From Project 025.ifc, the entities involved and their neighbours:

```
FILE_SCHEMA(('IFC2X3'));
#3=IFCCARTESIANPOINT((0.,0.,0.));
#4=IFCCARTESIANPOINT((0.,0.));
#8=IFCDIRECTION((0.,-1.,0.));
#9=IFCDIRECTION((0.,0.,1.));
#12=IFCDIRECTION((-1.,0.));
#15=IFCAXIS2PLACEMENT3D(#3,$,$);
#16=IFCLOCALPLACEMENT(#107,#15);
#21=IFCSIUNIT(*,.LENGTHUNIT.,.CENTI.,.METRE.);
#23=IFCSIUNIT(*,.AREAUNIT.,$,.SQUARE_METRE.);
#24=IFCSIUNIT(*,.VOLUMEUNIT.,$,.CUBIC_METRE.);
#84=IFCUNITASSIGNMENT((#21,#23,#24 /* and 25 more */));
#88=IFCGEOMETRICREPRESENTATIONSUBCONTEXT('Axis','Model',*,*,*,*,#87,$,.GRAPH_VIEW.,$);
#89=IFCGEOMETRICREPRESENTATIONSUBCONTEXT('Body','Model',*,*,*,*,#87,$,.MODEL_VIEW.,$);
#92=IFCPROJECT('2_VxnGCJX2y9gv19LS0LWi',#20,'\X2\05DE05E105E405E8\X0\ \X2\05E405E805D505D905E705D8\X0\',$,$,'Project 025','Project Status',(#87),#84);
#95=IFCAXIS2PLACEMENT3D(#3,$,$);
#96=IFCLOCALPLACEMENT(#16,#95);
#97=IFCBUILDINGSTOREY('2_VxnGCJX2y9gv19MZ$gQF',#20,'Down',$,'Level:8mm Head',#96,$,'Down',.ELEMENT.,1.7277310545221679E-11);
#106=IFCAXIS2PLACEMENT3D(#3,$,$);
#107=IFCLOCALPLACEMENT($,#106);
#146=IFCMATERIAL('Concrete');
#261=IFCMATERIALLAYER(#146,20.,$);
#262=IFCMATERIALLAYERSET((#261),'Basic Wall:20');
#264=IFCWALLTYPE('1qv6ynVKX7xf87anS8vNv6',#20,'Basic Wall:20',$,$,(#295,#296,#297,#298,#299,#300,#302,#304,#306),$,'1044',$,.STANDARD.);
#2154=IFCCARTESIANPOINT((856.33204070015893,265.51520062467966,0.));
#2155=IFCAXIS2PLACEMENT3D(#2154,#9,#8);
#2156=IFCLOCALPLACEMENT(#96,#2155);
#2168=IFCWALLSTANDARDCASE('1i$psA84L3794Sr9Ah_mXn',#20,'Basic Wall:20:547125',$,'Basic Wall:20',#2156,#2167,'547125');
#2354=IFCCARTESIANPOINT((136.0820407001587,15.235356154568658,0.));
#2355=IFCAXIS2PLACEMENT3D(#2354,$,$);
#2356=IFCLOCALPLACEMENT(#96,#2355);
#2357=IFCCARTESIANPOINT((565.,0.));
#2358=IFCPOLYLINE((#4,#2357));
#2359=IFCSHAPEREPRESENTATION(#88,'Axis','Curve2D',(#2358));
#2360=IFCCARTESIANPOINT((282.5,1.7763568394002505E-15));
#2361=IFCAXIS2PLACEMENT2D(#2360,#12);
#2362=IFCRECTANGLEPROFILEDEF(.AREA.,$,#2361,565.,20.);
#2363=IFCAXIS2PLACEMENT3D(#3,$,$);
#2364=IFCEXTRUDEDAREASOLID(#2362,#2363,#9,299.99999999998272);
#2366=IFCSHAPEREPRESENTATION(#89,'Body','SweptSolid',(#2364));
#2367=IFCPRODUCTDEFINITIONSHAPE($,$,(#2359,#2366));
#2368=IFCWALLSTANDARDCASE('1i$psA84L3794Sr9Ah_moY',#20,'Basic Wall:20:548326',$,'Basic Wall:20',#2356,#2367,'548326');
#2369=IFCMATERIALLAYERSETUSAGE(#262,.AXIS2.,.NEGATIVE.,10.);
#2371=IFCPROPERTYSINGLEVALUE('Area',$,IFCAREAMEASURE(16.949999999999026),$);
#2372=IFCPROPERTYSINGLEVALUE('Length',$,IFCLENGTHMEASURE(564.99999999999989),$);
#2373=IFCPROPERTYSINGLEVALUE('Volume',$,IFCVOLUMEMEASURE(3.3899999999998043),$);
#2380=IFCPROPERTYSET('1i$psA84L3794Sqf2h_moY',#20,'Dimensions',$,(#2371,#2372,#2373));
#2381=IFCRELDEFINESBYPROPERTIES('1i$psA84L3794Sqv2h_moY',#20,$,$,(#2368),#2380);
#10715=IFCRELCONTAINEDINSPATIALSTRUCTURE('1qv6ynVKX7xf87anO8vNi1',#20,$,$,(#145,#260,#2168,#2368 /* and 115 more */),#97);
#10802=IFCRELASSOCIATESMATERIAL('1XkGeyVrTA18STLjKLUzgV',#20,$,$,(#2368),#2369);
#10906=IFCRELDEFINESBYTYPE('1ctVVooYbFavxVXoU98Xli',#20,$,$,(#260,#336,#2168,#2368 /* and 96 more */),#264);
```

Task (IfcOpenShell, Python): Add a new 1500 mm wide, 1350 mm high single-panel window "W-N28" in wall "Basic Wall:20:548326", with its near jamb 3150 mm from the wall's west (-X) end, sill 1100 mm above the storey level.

```python
import numpy as np
import ifcopenshell
import ifcopenshell.api.feature
import ifcopenshell.api.geometry
import ifcopenshell.api.pset
import ifcopenshell.api.root
import ifcopenshell.api.spatial
import ifcopenshell.api.type
import ifcopenshell.geom
import ifcopenshell.util.element
import ifcopenshell.util.placement
import ifcopenshell.util.representation
import ifcopenshell.util.shape
import ifcopenshell.util.unit

model = ifcopenshell.open("Project 025.ifc")
unit_scale = ifcopenshell.util.unit.calculate_unit_scale(model)
area_scale = ifcopenshell.util.unit.calculate_unit_scale(model, "AREAUNIT")
volume_scale = ifcopenshell.util.unit.calculate_unit_scale(model, "VOLUMEUNIT")
settings = ifcopenshell.geom.settings()


def volume(element):
    """Net volume in cubic metres, openings subtracted."""
    shape = ifcopenshell.geom.create_shape(settings, element)
    return ifcopenshell.util.shape.get_volume(shape.geometry)


wall = model.by_id(2368)
storey = ifcopenshell.util.element.get_container(wall, ifc_class="IfcBuildingStorey")
context = ifcopenshell.util.representation.get_context(model, "Model", "Body", "MODEL_VIEW")
before = volume(wall)

width, height, from_end, sill = 1.5, 1.35, 3.15, 1.1  # metres

# The wall runs along its own X axis, and the end named is its -X end.
wall_shape = ifcopenshell.geom.create_shape(settings, wall)
x, y, z = ifcopenshell.util.shape.get_vertices(wall_shape.geometry).T
start = x.min() + from_end
face, thickness = float(y.min()), float(y.max() - y.min())
wall_matrix = ifcopenshell.util.placement.get_local_placement(wall.ObjectPlacement)
level = ifcopenshell.util.placement.get_local_placement(storey.ObjectPlacement)[2, 3]


def in_wall(x, y):
    """Placement at x, y metres in the wall's axes, at sill height."""
    matrix = wall_matrix.copy()
    matrix[:, 3] = wall_matrix @ np.array([x / unit_scale, y / unit_scale, 0.0, 1.0])
    matrix[2, 3] = level + sill / unit_scale
    return matrix


# Opening: a box that overshoots both wall faces by 50 mm.
opening = ifcopenshell.api.root.create_entity(model, ifc_class="IfcOpeningElement")
box = ifcopenshell.api.geometry.add_wall_representation(
    model, context=context, length=width, height=height, thickness=thickness + 0.1
)
ifcopenshell.api.geometry.assign_representation(model, product=opening, representation=box)
ifcopenshell.api.geometry.edit_object_placement(model, product=opening, matrix=in_wall(start, face - 0.05), is_si=False)
ifcopenshell.api.feature.add_feature(model, feature=opening, element=wall)

window = ifcopenshell.api.root.create_entity(model, ifc_class="IfcWindow", name="W-N28")
window.OverallWidth, window.OverallHeight = width / unit_scale, height / unit_scale
body = ifcopenshell.api.geometry.add_window_representation(
    model,
    context=context,
    overall_width=window.OverallWidth,
    overall_height=window.OverallHeight,
    partition_type="SINGLE_PANEL",
)
ifcopenshell.api.geometry.assign_representation(model, product=window, representation=body)
ifcopenshell.api.spatial.assign_container(model, products=[window], relating_structure=storey)
fills = ifcopenshell.api.feature.add_filling(model, opening=opening, element=window)
fills.OwnerHistory = window.OwnerHistory  # required in IFC2X3

# IFC2X3 keeps the operation on the window style.
style = ifcopenshell.api.root.create_entity(model, ifc_class="IfcWindowStyle", name="W-N28")
style.OperationType, style.ConstructionType = "SINGLE_PANEL", "NOTDEFINED"
style.ParameterTakesPrecedence = style.Sizeable = False
ifcopenshell.api.type.assign_type(model, related_objects=[window], relating_type=style)

# Centre the window in the wall's thickness.
ifcopenshell.api.geometry.edit_object_placement(model, product=window, matrix=in_wall(start, face), is_si=False)
window_shape = ifcopenshell.geom.create_shape(settings, window)
depth = ifcopenshell.util.shape.get_vertices(window_shape.geometry)[:, 1]
offset = face + thickness / 2 - (depth.min() + depth.max()) / 2
ifcopenshell.api.geometry.edit_object_placement(model, product=window, matrix=in_wall(start, offset), is_si=False)

after = volume(wall)

# Update the wall's stored quantities.
pset = model.by_id(ifcopenshell.util.element.get_pset(wall, "Dimensions", should_inherit=False)["id"])
ifcopenshell.api.pset.edit_pset(model, pset=pset, properties={
    "Area": model.create_entity("IfcAreaMeasure", after / thickness / area_scale),
    "Volume": model.create_entity("IfcVolumeMeasure", after / volume_scale),
})

print(f"wall volume {before:.3f} -> {after:.3f} m3")

model.write("Project 025-out.ifc")
```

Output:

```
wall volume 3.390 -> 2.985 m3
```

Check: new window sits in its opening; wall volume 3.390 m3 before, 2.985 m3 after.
